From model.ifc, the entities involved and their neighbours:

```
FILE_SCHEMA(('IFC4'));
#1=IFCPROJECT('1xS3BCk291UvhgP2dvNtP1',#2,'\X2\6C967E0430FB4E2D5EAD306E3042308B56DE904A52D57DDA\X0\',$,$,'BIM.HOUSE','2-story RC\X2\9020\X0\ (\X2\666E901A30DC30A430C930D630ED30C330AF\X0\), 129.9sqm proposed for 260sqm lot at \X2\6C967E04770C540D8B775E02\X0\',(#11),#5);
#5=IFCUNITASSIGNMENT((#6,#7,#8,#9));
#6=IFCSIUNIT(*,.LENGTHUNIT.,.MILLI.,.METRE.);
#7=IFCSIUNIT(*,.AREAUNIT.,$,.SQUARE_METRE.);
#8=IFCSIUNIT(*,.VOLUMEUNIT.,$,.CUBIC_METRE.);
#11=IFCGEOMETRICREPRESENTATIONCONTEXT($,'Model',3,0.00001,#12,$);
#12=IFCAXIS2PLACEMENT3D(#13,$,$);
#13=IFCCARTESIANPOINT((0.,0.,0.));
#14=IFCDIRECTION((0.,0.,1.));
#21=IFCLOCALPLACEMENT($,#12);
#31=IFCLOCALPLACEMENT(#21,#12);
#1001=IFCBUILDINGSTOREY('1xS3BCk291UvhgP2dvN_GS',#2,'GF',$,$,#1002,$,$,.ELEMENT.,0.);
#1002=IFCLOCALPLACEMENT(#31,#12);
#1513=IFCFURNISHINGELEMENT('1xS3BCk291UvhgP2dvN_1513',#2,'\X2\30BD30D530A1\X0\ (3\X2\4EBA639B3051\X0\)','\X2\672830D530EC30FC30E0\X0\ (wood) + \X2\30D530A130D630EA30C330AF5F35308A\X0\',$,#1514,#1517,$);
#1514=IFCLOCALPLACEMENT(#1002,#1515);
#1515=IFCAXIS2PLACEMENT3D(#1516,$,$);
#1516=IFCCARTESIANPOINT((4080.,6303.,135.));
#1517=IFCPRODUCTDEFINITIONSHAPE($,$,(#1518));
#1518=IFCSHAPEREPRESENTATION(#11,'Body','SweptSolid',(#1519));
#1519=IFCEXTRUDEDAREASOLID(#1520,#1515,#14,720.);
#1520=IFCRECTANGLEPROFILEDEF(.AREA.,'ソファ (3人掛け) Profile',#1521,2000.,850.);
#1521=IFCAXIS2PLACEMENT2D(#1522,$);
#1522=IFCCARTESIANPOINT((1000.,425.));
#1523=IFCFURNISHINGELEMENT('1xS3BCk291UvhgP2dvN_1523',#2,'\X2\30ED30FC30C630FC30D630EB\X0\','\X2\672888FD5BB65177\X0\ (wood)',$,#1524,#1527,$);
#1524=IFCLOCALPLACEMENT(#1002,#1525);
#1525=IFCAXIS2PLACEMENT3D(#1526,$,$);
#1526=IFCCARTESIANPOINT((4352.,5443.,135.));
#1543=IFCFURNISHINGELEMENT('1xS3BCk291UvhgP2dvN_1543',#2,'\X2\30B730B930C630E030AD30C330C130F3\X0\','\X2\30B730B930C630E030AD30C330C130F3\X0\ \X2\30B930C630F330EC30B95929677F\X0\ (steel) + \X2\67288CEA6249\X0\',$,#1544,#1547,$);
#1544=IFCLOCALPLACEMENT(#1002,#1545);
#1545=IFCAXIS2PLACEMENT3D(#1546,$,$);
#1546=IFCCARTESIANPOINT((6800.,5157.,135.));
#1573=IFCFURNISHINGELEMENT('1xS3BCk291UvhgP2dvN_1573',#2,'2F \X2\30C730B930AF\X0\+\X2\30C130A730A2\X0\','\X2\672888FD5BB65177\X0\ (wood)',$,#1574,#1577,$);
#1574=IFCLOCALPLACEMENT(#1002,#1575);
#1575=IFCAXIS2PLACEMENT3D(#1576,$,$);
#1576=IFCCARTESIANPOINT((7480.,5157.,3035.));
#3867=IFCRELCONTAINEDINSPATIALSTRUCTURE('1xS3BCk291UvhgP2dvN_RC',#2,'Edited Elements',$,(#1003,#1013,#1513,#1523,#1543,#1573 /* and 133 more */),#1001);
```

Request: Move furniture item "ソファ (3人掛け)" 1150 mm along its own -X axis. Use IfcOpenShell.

```python
import ifcopenshell
import ifcopenshell.api.geometry
import ifcopenshell.util.placement

model = ifcopenshell.open("model.ifc")

item = model.by_guid("1xS3BCk291UvhgP2dvN_1513")
matrix = ifcopenshell.util.placement.get_local_placement(item.ObjectPlacement)
matrix[:3, 3] -= matrix[:3, 0] * 1150.0
ifcopenshell.api.geometry.edit_object_placement(model, product=item, matrix=matrix, is_si=False)

print(ifcopenshell.util.placement.get_local_placement(item.ObjectPlacement).round(3) + 0.0)

model.write("model_rev.ifc")
```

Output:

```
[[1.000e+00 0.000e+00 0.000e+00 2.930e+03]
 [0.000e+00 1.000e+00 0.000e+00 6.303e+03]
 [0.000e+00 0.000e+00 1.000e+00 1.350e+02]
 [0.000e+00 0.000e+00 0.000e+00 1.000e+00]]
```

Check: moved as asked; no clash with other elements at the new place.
